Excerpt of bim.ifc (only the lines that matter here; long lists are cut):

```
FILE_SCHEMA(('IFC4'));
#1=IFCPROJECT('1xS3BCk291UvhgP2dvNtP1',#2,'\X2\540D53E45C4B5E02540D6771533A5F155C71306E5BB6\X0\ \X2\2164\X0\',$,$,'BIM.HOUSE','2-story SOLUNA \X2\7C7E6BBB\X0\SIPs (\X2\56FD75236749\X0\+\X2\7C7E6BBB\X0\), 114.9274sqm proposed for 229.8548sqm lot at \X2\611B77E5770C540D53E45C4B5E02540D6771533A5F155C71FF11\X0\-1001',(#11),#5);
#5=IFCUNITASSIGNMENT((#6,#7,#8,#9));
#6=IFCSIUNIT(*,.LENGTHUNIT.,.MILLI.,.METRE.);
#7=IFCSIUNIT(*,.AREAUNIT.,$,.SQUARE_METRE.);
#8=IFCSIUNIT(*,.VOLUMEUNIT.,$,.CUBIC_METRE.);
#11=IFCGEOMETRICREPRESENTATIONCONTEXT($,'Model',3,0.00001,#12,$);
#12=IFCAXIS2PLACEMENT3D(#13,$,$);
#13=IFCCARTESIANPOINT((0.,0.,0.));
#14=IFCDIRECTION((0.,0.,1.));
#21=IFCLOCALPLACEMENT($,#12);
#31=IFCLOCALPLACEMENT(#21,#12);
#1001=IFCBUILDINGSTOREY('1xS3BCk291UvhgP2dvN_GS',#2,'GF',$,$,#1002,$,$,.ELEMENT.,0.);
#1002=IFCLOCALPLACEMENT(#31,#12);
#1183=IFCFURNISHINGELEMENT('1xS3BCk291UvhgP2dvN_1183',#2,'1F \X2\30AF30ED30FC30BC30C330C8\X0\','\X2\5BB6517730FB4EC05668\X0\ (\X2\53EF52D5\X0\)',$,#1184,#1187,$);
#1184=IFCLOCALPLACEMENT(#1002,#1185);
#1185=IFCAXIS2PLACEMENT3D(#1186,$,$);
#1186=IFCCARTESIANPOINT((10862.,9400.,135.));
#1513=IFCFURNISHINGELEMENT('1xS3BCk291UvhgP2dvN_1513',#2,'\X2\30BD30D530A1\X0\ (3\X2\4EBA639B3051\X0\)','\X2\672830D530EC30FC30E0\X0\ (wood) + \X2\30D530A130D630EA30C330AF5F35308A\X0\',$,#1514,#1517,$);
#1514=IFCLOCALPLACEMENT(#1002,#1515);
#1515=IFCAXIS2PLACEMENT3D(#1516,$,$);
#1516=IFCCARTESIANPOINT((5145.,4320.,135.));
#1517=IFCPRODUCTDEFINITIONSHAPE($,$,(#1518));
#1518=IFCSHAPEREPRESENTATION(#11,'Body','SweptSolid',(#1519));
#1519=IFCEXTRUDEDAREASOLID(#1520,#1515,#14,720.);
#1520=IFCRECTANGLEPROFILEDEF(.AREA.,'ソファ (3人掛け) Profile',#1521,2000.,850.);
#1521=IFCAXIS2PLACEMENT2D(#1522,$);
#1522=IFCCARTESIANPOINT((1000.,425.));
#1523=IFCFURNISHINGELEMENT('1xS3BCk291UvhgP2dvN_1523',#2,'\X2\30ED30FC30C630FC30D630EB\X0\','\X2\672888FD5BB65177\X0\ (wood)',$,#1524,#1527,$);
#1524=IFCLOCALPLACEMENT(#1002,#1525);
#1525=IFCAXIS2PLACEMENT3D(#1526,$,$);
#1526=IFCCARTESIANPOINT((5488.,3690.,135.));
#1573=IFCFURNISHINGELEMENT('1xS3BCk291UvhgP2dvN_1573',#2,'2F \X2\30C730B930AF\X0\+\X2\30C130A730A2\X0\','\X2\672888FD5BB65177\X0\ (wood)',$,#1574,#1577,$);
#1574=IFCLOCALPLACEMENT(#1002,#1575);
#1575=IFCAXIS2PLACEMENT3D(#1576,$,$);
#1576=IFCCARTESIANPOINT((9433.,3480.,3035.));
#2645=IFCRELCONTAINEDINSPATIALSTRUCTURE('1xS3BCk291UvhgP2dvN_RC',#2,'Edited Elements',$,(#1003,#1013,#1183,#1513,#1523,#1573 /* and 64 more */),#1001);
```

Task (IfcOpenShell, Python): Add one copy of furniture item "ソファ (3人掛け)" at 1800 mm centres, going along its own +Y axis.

```python
import ifcopenshell
import ifcopenshell.api.geometry
import ifcopenshell.api.root
import ifcopenshell.util.element
import ifcopenshell.util.placement
import ifcopenshell.util.unit

model = ifcopenshell.open("bim.ifc")
unit_scale = ifcopenshell.util.unit.calculate_unit_scale(model)


def reuse_history(source, copy):
    """copy_class also copies each property set's owner history, people and application; keep the originals."""
    for rel in copy.IsDefinedBy:
        if rel.is_a("IfcRelDefinesByProperties") and (history := rel.RelatingPropertyDefinition.OwnerHistory):
            rel.RelatingPropertyDefinition.OwnerHistory = source.OwnerHistory
            ifcopenshell.util.element.remove_deep2(model, history)


source = model.by_guid("1xS3BCk291UvhgP2dvN_1513")
base = ifcopenshell.util.placement.get_local_placement(source.ObjectPlacement)
step = base[:3, 1] * 1.8 / unit_scale

for i in range(1, 2):
    copy = ifcopenshell.api.root.copy_class(model, product=source)
    copy.Representation = ifcopenshell.util.element.copy_deep(
        model, source.Representation, exclude=["IfcGeometricRepresentationContext", "IfcRepresentationMap"]
    )
    reuse_history(source, copy)
    matrix = base.copy()
    matrix[:3, 3] += i * step
    print("added at", matrix[:3, 3].round(3) + 0.0)
    ifcopenshell.api.geometry.edit_object_placement(model, product=copy, matrix=matrix, is_si=False)

model.write("bim_updated.ifc")
```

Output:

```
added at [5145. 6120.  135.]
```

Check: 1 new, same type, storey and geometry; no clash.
